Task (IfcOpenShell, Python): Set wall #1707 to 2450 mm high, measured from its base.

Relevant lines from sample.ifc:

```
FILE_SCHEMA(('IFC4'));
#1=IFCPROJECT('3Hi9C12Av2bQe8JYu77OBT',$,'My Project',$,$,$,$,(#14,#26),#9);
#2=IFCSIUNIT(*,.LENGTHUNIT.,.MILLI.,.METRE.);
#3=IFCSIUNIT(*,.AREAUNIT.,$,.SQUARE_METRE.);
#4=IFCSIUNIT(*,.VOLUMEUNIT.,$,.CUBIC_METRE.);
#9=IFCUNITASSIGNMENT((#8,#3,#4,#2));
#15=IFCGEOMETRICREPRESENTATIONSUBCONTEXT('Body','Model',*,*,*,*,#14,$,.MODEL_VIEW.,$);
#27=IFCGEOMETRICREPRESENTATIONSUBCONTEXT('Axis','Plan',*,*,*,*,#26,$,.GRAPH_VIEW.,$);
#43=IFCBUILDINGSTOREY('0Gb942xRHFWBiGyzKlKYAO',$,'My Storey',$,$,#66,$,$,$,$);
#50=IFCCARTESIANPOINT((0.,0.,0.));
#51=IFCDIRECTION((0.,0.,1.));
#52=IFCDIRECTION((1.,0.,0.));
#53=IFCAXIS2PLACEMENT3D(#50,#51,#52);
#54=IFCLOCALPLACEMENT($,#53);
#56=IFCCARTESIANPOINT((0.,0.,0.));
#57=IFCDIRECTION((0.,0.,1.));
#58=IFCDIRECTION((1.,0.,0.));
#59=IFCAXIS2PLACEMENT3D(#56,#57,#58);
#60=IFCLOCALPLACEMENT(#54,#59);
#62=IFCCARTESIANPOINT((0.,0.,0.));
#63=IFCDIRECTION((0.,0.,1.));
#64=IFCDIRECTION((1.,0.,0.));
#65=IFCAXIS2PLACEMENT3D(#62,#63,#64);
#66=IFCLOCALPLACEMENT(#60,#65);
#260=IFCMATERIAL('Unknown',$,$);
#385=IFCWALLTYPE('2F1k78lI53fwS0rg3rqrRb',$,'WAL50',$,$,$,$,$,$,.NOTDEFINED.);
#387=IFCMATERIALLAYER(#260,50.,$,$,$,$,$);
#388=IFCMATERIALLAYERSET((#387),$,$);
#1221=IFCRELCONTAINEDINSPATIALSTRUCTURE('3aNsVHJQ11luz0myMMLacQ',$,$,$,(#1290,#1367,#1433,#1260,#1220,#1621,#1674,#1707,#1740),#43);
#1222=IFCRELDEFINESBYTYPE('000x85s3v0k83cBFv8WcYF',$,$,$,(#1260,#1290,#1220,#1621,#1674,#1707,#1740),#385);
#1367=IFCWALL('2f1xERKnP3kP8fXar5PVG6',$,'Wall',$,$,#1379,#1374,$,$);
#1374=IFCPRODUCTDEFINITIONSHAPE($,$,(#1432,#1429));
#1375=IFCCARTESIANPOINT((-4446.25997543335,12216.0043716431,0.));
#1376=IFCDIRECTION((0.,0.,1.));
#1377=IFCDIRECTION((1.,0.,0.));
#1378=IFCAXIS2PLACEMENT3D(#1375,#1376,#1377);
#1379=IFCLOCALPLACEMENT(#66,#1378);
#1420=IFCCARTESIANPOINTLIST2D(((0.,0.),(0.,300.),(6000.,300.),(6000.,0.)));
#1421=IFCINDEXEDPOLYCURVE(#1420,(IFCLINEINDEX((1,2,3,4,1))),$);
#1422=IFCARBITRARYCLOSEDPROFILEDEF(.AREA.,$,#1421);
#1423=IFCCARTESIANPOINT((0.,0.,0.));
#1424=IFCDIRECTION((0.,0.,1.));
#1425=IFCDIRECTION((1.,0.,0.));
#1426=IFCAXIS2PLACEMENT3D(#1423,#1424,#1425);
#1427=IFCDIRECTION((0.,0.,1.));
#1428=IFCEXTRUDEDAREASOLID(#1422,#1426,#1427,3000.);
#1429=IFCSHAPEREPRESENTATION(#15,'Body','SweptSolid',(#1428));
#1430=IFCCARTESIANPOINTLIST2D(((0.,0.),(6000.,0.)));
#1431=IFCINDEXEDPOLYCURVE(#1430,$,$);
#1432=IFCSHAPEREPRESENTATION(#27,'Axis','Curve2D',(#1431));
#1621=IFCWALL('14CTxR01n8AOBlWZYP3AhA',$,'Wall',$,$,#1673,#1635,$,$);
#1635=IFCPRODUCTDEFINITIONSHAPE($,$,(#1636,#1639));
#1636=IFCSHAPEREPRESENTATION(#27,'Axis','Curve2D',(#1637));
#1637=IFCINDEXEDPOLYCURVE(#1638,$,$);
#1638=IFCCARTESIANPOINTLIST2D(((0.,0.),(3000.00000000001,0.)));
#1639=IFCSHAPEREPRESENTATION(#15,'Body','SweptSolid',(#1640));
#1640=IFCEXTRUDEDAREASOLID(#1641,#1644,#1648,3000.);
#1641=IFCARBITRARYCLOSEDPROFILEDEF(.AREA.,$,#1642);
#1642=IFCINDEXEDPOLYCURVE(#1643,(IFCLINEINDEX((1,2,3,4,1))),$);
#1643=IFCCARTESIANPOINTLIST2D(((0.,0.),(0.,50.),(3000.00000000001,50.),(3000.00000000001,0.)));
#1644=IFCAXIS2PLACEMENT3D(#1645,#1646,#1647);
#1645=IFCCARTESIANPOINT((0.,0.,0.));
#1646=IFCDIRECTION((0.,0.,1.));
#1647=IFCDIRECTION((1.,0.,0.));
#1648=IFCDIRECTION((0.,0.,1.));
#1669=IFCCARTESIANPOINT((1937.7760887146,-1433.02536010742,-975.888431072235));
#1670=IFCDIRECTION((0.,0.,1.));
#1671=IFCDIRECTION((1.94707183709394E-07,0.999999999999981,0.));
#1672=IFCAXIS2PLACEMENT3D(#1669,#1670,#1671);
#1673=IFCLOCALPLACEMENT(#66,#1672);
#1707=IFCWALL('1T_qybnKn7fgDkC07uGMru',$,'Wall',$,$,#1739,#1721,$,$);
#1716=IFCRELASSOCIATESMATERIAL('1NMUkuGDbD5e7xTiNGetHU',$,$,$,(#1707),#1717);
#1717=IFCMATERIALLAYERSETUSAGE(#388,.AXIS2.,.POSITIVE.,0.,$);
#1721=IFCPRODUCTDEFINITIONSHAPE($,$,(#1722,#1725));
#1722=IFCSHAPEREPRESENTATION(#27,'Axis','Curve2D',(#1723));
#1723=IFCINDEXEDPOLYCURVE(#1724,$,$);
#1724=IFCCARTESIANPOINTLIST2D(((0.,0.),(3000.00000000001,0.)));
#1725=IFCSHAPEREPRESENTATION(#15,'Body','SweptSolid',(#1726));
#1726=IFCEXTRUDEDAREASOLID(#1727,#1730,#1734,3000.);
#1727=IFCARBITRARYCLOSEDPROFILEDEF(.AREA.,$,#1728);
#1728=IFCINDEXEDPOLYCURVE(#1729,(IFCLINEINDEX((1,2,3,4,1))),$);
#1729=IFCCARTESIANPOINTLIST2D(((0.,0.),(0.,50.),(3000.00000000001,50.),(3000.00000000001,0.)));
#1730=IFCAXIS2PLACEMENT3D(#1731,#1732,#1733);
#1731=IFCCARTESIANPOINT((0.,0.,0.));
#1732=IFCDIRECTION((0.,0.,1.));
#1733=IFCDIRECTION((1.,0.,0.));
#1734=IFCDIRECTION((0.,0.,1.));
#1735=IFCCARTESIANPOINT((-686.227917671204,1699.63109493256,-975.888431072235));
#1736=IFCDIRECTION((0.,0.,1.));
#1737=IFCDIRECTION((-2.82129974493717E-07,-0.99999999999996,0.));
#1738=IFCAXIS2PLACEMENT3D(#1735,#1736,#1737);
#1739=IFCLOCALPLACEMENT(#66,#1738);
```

```python
import ifcopenshell
import ifcopenshell.geom
import ifcopenshell.util.representation
import ifcopenshell.util.shape

model = ifcopenshell.open("sample.ifc")
settings = ifcopenshell.geom.settings()


def volume(element):
    """Net volume in cubic metres, openings subtracted."""
    shape = ifcopenshell.geom.create_shape(settings, element)
    return ifcopenshell.util.shape.get_volume(shape.geometry)


wall = model.by_id(1707)
before = volume(wall)

body = ifcopenshell.util.representation.get_representation(wall, "Model", "Body")
solid = body.Items[0]
old_height = solid.Depth
solid.Depth = 2450.0
after = volume(wall)

print(f"height {old_height:g} -> {solid.Depth:g}, volume {before:.3f} -> {after:.3f} m3")

model.write("sample_rev.ifc")
```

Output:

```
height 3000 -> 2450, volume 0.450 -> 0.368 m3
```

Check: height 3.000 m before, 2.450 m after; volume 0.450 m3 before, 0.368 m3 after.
